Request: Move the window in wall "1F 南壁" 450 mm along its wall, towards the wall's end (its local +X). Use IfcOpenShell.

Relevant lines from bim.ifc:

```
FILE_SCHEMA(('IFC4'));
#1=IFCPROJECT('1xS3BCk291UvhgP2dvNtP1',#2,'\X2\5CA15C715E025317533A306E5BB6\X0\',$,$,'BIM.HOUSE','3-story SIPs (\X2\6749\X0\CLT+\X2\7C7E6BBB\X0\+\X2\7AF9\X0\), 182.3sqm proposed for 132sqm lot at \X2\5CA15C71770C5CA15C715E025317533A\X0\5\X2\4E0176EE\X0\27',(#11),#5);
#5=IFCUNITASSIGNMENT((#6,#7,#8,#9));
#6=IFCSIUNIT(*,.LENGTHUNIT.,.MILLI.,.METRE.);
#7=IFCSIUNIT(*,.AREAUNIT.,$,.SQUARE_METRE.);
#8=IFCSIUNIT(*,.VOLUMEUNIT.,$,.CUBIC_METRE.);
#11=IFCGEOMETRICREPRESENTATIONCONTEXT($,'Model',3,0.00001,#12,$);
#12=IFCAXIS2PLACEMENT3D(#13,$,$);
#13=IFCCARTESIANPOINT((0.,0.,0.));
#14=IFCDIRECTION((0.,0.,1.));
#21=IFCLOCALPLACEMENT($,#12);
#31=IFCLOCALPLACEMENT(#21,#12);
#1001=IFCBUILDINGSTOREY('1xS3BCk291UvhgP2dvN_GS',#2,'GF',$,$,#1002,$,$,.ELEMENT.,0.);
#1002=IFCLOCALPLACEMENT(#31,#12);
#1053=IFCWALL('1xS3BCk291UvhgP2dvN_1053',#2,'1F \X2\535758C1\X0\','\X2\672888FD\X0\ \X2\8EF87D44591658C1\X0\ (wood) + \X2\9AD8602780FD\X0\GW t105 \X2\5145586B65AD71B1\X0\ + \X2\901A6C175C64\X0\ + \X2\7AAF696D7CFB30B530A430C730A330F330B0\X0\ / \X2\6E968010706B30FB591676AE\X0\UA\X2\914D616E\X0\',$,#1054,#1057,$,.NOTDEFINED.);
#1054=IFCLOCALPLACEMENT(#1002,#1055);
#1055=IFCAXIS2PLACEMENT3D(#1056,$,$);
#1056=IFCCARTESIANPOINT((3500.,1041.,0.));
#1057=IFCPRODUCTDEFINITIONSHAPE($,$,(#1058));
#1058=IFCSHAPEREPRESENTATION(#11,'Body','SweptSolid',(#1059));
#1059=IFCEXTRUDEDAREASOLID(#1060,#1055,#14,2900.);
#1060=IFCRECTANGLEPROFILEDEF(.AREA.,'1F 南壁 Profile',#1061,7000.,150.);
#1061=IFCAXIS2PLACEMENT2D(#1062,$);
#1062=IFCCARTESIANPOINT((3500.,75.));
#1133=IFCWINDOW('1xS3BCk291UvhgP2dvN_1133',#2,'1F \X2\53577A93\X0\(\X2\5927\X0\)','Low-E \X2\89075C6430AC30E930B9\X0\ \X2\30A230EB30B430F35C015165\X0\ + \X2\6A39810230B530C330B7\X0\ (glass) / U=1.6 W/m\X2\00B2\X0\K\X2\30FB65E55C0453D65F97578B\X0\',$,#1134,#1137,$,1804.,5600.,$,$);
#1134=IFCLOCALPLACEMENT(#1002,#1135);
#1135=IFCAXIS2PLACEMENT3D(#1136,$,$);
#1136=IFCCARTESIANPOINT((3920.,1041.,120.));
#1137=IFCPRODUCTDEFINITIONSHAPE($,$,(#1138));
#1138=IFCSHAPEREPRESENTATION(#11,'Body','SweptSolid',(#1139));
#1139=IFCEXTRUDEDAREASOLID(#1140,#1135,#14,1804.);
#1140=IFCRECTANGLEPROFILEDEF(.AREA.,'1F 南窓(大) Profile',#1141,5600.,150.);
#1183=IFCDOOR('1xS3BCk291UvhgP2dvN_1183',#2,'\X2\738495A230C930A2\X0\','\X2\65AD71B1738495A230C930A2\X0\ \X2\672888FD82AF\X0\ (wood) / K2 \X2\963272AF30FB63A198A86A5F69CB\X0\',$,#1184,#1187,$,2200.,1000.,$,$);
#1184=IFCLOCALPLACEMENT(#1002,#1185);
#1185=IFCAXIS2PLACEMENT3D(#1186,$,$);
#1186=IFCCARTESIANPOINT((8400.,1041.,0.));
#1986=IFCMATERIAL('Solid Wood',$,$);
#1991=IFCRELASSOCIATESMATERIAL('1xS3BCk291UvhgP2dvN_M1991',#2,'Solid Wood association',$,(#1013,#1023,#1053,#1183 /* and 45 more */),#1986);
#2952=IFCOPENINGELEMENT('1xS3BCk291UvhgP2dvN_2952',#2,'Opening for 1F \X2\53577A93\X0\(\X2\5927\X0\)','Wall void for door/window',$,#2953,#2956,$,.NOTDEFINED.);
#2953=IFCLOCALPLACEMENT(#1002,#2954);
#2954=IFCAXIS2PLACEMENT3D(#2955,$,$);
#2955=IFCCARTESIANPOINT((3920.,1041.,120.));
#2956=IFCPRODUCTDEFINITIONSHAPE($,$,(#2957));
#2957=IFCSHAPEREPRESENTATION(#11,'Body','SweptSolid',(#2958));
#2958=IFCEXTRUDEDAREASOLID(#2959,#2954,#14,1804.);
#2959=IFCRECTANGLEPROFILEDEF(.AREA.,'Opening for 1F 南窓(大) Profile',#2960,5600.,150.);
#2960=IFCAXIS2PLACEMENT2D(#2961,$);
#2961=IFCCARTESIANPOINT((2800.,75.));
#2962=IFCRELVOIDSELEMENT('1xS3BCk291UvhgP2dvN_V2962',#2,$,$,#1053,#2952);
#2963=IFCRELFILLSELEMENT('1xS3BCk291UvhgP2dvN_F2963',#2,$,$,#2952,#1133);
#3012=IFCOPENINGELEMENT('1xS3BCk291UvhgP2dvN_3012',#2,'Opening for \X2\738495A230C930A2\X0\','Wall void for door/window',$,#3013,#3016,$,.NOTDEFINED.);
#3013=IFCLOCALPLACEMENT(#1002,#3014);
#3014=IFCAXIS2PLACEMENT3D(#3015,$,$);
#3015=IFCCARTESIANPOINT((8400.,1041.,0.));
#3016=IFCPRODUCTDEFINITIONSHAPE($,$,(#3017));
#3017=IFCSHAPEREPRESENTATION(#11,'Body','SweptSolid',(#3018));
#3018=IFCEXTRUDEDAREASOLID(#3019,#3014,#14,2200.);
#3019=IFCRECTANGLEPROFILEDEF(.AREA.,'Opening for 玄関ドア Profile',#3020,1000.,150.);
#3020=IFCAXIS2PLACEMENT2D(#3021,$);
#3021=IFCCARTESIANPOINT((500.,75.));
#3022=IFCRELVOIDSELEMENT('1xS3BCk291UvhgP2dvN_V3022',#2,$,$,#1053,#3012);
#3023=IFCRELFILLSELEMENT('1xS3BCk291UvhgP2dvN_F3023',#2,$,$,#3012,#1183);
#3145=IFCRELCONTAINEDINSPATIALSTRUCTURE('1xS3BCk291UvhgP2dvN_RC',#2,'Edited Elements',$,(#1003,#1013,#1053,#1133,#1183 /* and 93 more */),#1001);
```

```python
import ifcopenshell
import ifcopenshell.api.geometry
import ifcopenshell.util.placement

model = ifcopenshell.open("bim.ifc")

window = model.by_guid("1xS3BCk291UvhgP2dvN_1133")
opening = window.FillsVoids[0].RelatingOpeningElement
wall = opening.VoidsElements[0].RelatingBuildingElement

wall_matrix = ifcopenshell.util.placement.get_local_placement(wall.ObjectPlacement)
shift = wall_matrix[:3, 0] * 450.0
before = ifcopenshell.util.placement.get_local_placement(window.ObjectPlacement)[:3, 3].copy()

# The window is not placed relative to its opening, so move both.
for product in (opening, window):
    matrix = ifcopenshell.util.placement.get_local_placement(product.ObjectPlacement)
    matrix[:3, 3] += shift
    ifcopenshell.api.geometry.edit_object_placement(model, product=product, matrix=matrix, is_si=False)

after = ifcopenshell.util.placement.get_local_placement(window.ObjectPlacement)[:3, 3]
print("window moved by", (after - before).round(3) + 0.0)

model.write("bim_v2.ifc")
```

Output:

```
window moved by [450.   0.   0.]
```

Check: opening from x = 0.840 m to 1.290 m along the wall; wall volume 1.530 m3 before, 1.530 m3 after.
